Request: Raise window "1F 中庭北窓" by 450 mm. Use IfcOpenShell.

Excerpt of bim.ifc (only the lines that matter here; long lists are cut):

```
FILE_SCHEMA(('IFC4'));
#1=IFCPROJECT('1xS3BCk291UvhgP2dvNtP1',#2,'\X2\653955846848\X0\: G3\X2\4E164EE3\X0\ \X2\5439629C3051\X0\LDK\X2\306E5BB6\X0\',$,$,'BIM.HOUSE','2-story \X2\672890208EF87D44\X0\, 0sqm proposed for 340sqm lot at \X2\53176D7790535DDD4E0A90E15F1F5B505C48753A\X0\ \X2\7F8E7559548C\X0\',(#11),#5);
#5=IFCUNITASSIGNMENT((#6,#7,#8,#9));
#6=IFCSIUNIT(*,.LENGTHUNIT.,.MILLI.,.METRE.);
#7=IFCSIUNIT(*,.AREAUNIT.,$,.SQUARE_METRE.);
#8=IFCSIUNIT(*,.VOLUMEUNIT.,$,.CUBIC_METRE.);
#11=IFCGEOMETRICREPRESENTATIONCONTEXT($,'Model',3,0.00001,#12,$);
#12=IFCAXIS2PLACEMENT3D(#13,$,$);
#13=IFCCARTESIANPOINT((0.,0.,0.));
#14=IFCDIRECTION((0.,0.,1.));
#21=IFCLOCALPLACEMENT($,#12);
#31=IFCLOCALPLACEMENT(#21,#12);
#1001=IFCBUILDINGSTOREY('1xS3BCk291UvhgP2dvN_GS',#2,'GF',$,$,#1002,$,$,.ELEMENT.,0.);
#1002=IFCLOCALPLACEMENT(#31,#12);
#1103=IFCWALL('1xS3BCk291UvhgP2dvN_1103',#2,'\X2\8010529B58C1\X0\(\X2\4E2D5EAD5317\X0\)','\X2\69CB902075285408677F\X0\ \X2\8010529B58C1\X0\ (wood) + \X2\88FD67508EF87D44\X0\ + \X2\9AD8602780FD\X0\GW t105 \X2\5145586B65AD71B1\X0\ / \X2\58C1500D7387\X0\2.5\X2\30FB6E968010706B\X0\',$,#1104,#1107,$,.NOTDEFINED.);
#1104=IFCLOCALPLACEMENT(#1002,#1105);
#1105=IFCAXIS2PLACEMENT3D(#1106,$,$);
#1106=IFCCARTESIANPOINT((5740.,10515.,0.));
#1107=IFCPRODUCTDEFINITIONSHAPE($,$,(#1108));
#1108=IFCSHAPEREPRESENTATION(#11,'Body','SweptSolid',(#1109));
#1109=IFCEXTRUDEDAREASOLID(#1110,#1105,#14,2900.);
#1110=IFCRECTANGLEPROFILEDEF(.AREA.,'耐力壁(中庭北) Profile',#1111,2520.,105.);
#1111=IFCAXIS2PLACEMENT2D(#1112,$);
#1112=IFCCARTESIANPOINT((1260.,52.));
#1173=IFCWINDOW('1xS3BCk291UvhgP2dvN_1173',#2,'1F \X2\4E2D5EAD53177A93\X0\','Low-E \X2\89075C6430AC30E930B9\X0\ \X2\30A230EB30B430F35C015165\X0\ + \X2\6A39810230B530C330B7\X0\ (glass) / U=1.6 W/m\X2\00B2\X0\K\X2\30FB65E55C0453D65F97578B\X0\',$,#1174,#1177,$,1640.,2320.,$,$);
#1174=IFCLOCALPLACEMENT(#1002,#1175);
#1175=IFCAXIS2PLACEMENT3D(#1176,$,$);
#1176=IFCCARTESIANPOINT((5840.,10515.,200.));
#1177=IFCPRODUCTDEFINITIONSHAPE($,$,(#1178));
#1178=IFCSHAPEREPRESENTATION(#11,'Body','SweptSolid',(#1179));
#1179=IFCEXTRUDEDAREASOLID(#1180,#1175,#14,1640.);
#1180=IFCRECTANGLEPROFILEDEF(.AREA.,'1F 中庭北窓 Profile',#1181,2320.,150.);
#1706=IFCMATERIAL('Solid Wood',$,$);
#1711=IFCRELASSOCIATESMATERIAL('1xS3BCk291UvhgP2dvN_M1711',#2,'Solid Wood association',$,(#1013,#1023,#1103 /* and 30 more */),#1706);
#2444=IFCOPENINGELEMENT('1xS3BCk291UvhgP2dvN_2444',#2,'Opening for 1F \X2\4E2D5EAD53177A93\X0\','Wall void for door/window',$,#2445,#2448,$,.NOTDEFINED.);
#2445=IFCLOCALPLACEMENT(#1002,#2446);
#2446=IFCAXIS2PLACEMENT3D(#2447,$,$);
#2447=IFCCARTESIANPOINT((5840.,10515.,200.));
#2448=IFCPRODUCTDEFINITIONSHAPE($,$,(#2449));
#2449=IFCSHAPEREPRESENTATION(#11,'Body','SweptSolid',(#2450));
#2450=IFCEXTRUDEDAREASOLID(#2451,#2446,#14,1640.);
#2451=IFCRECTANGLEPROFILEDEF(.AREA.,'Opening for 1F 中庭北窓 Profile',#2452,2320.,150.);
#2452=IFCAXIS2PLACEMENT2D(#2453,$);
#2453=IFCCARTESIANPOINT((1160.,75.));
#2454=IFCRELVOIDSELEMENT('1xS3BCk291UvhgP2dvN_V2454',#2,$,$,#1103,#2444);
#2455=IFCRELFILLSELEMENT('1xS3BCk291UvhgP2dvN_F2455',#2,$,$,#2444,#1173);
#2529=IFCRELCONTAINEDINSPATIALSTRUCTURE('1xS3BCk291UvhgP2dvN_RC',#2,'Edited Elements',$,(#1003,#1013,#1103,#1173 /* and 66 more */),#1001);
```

```python
import numpy as np
import ifcopenshell
import ifcopenshell.api.geometry
import ifcopenshell.util.placement
import ifcopenshell.util.unit

model = ifcopenshell.open("bim.ifc")
unit_scale = ifcopenshell.util.unit.calculate_unit_scale(model)

window = model.by_guid("1xS3BCk291UvhgP2dvN_1173")
opening = window.FillsVoids[0].RelatingOpeningElement
dz = 450.0

shift = np.array([0.0, 0.0, dz])
# The window is not placed relative to its opening, so move both.
for product in (opening, window):
    matrix = ifcopenshell.util.placement.get_local_placement(product.ObjectPlacement)
    matrix[:3, 3] += shift
    ifcopenshell.api.geometry.edit_object_placement(model, product=product, matrix=matrix, is_si=False)

print(f"moved by {dz * unit_scale:+.3f} m")

model.write("bim_v2.ifc")
```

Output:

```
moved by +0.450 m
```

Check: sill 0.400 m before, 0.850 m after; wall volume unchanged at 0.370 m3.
